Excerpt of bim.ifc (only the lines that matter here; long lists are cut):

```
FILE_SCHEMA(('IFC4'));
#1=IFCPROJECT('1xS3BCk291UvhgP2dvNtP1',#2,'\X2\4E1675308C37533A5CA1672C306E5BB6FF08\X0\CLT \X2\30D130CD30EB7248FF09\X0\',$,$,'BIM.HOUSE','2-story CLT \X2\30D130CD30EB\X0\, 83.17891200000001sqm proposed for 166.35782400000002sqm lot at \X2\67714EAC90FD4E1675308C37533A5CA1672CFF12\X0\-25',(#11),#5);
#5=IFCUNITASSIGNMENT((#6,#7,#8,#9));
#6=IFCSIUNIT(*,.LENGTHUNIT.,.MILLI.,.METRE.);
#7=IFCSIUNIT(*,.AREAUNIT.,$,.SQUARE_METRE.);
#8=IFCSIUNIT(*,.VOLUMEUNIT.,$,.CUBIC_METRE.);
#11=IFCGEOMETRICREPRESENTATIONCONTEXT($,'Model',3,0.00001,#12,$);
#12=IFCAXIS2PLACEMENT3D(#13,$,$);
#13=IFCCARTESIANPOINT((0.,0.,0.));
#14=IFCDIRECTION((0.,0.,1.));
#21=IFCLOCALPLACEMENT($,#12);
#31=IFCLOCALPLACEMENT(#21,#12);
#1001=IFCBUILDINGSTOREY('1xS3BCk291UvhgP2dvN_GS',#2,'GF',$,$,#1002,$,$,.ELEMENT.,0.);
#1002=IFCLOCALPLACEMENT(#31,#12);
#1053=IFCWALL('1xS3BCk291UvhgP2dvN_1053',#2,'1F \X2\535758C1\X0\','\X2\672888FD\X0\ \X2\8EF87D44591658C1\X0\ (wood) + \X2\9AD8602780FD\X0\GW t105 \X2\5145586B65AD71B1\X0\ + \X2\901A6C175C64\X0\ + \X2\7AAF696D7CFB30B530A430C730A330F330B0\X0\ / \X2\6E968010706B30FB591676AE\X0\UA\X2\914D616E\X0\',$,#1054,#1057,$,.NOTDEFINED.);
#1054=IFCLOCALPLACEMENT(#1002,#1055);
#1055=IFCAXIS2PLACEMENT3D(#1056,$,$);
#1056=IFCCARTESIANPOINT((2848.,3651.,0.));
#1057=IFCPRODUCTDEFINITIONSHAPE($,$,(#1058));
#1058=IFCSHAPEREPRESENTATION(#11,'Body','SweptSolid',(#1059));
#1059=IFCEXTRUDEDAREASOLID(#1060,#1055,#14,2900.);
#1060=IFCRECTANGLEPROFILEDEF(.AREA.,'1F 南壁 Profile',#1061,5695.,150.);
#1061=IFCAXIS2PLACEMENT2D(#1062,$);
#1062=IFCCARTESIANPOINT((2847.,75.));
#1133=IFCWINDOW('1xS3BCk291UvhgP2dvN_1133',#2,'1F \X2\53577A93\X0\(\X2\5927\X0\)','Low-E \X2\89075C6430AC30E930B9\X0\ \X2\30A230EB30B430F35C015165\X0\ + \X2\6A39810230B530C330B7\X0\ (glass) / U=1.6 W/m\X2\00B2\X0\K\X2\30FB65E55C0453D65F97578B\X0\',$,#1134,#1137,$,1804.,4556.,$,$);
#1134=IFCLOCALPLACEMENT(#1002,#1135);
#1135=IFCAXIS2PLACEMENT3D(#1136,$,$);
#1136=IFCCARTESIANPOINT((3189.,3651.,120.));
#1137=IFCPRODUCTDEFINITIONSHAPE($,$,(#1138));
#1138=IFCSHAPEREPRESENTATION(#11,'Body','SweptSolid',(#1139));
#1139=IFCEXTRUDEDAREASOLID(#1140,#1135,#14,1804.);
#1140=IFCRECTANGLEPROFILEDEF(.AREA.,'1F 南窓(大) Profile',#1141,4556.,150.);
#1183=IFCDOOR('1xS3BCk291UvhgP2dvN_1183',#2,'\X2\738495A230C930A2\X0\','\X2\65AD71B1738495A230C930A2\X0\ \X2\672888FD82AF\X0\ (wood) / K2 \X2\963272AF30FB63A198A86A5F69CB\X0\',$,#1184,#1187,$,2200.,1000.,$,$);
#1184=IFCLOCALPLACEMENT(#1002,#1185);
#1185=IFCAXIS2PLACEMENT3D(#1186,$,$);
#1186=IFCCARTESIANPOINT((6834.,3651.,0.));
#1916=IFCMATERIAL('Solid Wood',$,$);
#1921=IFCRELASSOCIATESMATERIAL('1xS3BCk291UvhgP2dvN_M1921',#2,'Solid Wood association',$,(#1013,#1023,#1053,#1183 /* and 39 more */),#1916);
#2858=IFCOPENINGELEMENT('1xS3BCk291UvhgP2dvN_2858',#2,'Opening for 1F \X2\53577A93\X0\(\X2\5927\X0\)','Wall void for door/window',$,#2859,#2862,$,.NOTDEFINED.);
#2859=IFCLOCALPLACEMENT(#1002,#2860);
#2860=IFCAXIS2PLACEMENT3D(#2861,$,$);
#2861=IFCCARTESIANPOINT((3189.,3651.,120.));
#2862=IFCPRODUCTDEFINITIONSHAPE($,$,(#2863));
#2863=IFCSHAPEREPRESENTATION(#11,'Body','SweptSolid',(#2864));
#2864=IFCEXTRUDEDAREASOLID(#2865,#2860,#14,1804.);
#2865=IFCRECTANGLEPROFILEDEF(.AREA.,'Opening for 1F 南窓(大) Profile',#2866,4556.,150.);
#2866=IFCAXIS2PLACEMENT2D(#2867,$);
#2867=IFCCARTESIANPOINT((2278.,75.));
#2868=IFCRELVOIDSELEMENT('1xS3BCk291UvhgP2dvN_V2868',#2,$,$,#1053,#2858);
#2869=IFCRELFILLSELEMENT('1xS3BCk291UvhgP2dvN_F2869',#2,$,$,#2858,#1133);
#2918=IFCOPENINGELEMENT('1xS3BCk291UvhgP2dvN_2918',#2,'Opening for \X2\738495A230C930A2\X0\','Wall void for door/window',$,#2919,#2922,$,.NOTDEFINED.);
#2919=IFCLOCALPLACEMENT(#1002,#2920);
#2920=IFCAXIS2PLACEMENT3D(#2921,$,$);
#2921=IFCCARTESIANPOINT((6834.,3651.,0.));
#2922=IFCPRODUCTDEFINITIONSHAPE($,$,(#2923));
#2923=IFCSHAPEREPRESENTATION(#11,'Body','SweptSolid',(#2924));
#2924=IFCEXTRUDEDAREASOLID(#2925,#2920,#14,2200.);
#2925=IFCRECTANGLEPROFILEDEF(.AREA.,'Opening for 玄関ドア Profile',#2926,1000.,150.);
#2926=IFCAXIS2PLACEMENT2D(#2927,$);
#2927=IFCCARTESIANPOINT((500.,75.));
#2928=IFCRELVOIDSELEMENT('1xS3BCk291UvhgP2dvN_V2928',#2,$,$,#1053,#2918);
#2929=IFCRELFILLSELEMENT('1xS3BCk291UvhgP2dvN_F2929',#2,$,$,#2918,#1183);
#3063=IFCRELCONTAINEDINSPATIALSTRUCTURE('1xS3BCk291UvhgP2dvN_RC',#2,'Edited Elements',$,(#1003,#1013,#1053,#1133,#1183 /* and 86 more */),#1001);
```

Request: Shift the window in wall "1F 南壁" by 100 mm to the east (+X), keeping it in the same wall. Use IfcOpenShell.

```python
import ifcopenshell
import ifcopenshell.api.geometry
import ifcopenshell.util.placement
import ifcopenshell.util.unit

model = ifcopenshell.open("bim.ifc")
unit_scale = ifcopenshell.util.unit.calculate_unit_scale(model)

window = model.by_guid("1xS3BCk291UvhgP2dvN_1133")
opening = window.FillsVoids[0].RelatingOpeningElement
wall = opening.VoidsElements[0].RelatingBuildingElement

wall_matrix = ifcopenshell.util.placement.get_local_placement(wall.ObjectPlacement)
shift = wall_matrix[:3, 0] * 0.1 / unit_scale
before = ifcopenshell.util.placement.get_local_placement(window.ObjectPlacement)[:3, 3].copy()

# The window is not placed relative to its opening, so move both.
for product in (opening, window):
    matrix = ifcopenshell.util.placement.get_local_placement(product.ObjectPlacement)
    matrix[:3, 3] += shift
    ifcopenshell.api.geometry.edit_object_placement(model, product=product, matrix=matrix, is_si=False)

after = ifcopenshell.util.placement.get_local_placement(window.ObjectPlacement)[:3, 3]
print("window moved by", (after - before).round(3) + 0.0)

model.write("bim-out.ifc")
```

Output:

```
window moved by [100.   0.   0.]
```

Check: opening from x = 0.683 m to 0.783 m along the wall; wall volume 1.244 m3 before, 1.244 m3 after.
